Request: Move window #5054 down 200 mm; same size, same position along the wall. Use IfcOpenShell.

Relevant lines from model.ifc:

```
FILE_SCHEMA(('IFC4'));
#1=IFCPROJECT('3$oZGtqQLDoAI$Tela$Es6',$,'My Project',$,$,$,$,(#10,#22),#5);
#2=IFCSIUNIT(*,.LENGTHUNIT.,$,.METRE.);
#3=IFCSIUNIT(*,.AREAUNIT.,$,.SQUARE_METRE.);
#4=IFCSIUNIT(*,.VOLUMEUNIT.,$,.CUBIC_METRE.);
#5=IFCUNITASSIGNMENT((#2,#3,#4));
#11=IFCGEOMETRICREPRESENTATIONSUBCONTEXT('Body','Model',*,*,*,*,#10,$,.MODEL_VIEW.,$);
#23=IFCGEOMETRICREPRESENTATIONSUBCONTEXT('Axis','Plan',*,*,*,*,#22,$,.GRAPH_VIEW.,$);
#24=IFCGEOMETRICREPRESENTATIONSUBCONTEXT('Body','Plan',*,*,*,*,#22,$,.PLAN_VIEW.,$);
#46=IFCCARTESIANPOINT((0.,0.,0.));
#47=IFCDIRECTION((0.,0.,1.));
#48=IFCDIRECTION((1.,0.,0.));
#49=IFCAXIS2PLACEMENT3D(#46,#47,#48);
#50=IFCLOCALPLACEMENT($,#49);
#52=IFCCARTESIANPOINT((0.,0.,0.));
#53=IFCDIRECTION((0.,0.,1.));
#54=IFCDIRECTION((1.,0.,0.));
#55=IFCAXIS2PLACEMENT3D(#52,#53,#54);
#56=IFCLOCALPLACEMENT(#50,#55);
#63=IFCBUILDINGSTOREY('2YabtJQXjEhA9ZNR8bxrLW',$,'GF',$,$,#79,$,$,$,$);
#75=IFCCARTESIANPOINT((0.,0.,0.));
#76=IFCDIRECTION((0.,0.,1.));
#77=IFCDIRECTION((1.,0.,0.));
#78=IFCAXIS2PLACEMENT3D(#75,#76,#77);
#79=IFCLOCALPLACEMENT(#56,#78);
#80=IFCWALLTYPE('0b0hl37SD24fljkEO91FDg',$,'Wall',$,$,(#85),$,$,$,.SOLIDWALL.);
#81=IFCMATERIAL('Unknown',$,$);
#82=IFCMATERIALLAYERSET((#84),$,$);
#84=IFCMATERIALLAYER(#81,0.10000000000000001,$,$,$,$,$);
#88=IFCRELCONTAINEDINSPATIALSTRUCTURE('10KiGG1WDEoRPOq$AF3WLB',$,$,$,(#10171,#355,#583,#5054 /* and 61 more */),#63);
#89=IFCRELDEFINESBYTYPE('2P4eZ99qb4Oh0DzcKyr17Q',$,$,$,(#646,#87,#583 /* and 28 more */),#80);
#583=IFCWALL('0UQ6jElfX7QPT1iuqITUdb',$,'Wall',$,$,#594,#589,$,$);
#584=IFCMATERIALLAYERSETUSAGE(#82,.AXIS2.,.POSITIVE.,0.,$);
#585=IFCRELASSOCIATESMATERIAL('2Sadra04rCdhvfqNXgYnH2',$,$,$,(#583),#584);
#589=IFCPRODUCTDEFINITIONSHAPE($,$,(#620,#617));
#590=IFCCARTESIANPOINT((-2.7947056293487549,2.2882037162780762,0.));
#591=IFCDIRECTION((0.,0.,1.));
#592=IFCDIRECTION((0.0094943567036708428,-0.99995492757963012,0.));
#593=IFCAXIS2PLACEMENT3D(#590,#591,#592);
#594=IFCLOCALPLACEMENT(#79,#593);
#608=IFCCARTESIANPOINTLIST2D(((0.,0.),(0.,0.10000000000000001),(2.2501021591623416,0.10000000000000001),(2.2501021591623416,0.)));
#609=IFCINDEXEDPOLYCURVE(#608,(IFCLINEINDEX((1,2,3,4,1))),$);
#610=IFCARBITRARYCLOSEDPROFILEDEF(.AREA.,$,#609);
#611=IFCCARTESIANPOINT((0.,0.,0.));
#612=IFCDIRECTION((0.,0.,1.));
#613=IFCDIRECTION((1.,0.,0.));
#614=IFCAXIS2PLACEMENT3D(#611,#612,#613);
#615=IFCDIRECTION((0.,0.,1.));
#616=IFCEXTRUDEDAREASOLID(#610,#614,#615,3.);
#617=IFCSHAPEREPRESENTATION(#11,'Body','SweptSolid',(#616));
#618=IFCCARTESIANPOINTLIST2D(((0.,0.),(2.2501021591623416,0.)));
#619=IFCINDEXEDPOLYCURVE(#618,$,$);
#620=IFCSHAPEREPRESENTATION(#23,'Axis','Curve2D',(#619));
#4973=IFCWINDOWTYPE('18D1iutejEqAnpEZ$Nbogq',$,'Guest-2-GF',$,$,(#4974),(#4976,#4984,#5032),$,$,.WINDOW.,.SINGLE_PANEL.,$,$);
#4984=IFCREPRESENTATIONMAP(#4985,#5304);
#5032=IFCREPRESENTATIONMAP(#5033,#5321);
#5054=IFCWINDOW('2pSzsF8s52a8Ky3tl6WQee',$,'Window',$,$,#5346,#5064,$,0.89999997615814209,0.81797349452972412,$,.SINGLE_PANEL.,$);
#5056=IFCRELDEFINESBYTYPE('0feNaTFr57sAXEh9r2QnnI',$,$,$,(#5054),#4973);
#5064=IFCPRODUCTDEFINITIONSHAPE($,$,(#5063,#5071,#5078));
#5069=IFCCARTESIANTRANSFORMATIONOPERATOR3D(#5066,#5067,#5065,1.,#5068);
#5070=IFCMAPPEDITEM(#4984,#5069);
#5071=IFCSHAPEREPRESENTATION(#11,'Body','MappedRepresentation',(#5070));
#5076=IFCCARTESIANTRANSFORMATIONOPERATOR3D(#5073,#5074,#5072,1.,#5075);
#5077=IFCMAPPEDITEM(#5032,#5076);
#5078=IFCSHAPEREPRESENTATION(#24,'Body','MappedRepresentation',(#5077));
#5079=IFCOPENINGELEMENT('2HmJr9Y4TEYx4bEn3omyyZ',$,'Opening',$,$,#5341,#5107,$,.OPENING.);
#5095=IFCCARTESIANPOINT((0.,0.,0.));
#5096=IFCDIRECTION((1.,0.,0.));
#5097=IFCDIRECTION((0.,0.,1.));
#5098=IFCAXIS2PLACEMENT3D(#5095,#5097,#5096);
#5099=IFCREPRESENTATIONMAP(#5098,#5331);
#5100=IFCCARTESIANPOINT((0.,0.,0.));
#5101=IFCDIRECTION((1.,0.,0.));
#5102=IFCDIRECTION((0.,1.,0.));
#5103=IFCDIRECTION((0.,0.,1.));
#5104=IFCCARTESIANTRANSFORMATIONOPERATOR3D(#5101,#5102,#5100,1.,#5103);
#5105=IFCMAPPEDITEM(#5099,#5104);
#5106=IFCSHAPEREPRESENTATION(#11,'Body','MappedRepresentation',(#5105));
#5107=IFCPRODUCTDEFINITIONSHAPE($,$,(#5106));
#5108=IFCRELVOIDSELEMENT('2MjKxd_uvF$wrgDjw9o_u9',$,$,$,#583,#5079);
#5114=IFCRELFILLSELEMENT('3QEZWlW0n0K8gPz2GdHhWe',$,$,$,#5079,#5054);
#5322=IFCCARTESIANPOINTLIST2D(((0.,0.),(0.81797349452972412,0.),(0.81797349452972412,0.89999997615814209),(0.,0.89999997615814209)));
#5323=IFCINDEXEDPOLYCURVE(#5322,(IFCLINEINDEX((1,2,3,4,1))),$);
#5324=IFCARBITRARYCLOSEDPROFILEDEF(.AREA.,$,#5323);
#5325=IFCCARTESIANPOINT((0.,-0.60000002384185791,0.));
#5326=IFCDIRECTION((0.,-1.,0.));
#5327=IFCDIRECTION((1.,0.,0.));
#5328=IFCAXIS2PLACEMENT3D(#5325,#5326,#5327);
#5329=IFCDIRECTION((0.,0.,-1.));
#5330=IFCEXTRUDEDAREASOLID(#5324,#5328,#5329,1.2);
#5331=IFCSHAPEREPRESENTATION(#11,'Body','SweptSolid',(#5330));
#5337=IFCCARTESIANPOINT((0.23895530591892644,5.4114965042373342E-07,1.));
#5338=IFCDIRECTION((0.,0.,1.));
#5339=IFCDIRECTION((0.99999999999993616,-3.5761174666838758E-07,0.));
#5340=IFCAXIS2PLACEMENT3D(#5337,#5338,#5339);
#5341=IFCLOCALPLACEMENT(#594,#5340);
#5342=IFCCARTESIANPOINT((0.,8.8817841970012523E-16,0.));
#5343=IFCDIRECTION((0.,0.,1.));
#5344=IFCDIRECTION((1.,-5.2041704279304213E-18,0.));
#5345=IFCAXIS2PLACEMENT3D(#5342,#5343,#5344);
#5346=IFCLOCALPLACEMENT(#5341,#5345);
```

```python
import numpy as np
import ifcopenshell
import ifcopenshell.api.geometry
import ifcopenshell.util.placement
import ifcopenshell.util.unit

model = ifcopenshell.open("model.ifc")
unit_scale = ifcopenshell.util.unit.calculate_unit_scale(model)

window = model.by_guid("2pSzsF8s52a8Ky3tl6WQee")
opening = window.FillsVoids[0].RelatingOpeningElement
dz = -0.2

shift = np.array([0.0, 0.0, dz])
# The window is placed relative to its opening, so it follows when the opening moves.
matrix = ifcopenshell.util.placement.get_local_placement(opening.ObjectPlacement)
matrix[:3, 3] += shift
ifcopenshell.api.geometry.edit_object_placement(
    model, product=opening, matrix=matrix, is_si=False, should_transform_children=True
)

print(f"moved by {dz * unit_scale:+.3f} m")

model.write("model_updated.ifc")
```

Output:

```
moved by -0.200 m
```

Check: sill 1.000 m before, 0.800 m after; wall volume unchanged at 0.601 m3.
